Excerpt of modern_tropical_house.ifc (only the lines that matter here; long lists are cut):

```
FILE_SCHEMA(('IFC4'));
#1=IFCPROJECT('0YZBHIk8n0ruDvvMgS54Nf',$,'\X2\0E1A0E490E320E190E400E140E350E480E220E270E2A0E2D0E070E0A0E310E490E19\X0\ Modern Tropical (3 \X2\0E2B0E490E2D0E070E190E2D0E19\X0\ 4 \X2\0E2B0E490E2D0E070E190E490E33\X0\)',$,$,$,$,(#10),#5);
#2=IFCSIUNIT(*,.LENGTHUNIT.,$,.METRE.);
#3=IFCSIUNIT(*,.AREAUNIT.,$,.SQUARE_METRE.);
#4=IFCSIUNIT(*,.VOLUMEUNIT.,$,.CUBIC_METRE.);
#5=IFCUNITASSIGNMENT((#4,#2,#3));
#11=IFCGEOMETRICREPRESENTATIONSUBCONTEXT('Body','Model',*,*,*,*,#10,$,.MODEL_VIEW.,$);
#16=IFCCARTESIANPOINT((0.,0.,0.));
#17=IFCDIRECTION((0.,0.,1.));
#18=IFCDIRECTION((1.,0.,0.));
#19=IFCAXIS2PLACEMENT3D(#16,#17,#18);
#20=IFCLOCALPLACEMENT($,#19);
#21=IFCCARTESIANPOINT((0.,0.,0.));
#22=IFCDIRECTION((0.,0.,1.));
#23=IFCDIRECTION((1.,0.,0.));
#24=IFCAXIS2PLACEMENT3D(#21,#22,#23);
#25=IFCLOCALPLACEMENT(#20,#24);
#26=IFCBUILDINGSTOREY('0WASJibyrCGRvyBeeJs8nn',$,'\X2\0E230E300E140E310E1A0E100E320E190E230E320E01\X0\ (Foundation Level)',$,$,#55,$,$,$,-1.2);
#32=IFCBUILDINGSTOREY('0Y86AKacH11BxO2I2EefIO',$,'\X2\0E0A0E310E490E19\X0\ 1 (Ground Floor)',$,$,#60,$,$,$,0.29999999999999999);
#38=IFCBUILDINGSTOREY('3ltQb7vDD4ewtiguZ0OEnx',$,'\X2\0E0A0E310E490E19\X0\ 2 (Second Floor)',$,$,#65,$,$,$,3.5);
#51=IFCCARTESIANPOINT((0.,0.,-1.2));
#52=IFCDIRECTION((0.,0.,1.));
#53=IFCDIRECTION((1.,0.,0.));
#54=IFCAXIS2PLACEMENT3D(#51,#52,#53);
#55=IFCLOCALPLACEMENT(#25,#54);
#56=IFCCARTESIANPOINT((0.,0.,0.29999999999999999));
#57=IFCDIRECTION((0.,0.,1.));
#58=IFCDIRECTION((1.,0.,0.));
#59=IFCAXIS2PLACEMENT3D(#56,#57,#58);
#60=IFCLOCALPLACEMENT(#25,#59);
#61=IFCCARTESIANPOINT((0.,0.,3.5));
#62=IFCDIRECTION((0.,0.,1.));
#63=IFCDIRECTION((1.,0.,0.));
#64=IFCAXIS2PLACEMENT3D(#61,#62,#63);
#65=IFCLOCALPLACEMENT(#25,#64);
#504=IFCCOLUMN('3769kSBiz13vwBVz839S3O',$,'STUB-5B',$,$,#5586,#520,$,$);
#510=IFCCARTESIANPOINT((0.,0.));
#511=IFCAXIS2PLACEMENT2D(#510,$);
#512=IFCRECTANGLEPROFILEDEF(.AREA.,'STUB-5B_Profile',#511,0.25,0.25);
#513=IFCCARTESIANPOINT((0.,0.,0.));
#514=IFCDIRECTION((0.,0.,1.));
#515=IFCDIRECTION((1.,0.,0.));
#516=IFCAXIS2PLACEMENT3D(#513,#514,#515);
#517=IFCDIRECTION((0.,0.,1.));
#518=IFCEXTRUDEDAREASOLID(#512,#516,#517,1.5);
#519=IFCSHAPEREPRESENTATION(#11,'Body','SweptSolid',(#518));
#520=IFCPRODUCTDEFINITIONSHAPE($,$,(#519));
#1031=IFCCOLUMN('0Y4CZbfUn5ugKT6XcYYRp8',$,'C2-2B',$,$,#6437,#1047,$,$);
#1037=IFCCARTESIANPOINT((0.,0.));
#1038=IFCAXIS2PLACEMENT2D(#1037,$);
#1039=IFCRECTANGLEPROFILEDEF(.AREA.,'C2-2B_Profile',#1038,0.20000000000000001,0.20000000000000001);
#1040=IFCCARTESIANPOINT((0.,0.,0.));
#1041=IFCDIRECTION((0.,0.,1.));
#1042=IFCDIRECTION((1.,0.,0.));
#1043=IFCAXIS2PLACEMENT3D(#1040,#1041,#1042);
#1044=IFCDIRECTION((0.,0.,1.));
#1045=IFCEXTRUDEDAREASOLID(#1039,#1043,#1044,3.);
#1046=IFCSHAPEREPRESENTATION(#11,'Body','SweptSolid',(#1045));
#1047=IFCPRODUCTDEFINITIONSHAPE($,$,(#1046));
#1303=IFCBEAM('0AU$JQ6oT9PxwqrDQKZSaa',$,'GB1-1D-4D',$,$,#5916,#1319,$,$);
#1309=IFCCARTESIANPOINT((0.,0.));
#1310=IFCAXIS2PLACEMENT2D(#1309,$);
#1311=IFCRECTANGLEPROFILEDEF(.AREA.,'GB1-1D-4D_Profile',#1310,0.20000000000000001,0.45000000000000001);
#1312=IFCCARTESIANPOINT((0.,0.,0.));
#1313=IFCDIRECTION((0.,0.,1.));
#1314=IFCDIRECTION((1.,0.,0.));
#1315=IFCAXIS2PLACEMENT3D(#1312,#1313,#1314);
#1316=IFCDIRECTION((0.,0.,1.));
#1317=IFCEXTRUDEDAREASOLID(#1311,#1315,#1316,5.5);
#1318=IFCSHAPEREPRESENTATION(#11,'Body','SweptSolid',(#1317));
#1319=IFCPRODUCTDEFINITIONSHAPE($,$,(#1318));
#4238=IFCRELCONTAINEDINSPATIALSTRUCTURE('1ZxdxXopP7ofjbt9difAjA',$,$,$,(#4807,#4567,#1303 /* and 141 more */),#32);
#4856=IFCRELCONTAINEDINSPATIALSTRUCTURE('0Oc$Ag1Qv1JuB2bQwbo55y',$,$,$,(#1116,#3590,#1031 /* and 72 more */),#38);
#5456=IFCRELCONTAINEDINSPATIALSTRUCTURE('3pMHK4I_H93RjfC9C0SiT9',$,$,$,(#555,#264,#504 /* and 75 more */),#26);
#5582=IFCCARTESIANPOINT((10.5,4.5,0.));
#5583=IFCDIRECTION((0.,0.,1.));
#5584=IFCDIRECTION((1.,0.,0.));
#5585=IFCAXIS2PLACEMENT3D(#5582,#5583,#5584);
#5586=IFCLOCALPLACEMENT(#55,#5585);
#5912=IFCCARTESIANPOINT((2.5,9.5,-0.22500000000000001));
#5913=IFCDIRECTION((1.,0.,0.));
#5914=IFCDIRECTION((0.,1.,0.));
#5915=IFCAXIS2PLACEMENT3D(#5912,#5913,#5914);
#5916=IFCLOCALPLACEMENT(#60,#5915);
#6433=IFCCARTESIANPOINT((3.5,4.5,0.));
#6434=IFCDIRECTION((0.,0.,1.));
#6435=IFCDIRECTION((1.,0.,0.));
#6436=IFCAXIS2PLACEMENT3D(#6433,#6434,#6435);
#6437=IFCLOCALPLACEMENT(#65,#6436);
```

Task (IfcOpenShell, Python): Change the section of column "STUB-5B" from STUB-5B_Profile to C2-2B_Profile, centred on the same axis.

```python
import ifcopenshell
import ifcopenshell.util.element
import ifcopenshell.util.representation

model = ifcopenshell.open("modern_tropical_house.ifc")

member = model.by_id(504)
source = next(p for p in model.by_type("IfcRectangleProfileDef") if p.ProfileName == "C2-2B_Profile")

body = ifcopenshell.util.representation.get_representation(member, "Model", "Body")
solid = body.Items[0]
old_profile = solid.SweptArea

# Copy the section's sizes but keep this member's own profile position.
profile = ifcopenshell.util.element.copy(model, source)
profile.Position = old_profile.Position
solid.SweptArea = profile
if not model.get_total_inverses(old_profile):
    ifcopenshell.util.element.remove_deep2(model, old_profile)

print(solid.SweptArea)

model.write("modern_tropical_house_v2.ifc")
```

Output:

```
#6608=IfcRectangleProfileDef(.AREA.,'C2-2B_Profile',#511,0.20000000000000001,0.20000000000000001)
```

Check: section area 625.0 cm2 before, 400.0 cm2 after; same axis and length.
